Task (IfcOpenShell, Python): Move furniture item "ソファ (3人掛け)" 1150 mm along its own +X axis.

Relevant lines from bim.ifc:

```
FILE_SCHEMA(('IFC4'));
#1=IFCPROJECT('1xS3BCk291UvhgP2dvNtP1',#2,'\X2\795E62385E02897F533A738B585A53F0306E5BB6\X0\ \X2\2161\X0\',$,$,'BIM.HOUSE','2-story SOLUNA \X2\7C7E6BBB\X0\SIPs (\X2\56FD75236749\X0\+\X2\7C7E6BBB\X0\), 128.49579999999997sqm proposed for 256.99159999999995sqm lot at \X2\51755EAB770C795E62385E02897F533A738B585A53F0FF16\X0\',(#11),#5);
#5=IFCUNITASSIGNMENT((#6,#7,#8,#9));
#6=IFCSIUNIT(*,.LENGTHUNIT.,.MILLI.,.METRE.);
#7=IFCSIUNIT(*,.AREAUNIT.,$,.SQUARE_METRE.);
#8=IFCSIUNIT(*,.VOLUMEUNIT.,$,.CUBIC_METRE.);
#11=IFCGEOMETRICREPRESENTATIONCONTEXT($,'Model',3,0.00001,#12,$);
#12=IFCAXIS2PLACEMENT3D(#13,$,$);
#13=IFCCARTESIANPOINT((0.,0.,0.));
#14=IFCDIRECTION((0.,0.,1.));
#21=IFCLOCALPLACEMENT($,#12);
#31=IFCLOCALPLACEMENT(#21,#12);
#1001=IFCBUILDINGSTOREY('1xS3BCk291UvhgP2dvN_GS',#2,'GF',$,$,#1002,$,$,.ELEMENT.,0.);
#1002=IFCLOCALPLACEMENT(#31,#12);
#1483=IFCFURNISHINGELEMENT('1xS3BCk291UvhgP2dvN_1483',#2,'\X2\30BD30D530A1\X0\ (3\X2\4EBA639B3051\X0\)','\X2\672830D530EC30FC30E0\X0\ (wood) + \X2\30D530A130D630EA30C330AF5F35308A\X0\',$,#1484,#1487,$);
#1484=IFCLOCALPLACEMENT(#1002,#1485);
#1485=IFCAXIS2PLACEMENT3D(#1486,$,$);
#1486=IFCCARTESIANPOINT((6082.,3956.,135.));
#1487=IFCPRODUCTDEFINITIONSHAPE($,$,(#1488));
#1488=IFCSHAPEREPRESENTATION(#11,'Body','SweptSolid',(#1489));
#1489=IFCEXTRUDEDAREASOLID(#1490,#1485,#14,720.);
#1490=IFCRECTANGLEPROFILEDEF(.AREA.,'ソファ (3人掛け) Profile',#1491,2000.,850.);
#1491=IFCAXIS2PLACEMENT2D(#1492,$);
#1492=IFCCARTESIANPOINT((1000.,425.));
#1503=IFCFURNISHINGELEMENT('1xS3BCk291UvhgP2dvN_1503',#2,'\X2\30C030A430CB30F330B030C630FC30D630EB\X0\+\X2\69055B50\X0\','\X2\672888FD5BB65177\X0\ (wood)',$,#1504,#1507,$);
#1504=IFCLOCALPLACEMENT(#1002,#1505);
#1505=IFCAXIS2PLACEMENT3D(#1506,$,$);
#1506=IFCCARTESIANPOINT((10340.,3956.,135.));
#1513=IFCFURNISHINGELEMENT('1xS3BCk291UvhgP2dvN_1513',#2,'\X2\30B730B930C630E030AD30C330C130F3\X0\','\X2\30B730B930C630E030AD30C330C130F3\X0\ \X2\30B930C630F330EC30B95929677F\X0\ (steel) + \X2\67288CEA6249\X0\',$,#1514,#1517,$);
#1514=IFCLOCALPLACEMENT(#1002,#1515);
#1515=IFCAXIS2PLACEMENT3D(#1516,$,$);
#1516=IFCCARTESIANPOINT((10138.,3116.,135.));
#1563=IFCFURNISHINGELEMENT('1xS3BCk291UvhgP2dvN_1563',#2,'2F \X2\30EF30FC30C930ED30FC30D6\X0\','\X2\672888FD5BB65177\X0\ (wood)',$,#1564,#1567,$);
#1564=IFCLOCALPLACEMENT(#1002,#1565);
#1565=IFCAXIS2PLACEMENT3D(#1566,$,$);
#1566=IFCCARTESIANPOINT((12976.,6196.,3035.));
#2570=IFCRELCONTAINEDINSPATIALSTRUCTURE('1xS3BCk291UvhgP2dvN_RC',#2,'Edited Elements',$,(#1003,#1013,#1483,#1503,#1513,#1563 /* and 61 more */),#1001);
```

```python
import ifcopenshell
import ifcopenshell.api.geometry
import ifcopenshell.util.placement

model = ifcopenshell.open("bim.ifc")

item = model.by_id(1483)
matrix = ifcopenshell.util.placement.get_local_placement(item.ObjectPlacement)
matrix[:3, 3] += matrix[:3, 0] * 1150.0
ifcopenshell.api.geometry.edit_object_placement(model, product=item, matrix=matrix, is_si=False)

print(ifcopenshell.util.placement.get_local_placement(item.ObjectPlacement).round(3) + 0.0)

model.write("bim-out.ifc")
```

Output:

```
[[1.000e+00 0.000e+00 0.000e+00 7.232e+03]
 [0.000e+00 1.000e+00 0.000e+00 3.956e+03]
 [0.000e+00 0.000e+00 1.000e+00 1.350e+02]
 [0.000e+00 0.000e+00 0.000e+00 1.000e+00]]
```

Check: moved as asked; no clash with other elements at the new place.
